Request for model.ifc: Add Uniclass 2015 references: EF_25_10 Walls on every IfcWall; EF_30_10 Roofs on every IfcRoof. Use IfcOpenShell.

First a look at what the model holds.

```python
import ifcopenshell

model = ifcopenshell.open("model.ifc")
print(model.schema)
print("classifications:", [c.Name for c in model.by_type("IfcClassification")])
for ifc_class in ("IfcDoor", "IfcRoof", "IfcStair", "IfcWall", "IfcWindow"):
    print(ifc_class, len(model.by_type(ifc_class)))
```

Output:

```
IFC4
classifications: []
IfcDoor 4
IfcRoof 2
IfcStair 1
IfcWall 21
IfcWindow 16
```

```python
import ifcopenshell
import ifcopenshell.api.classification

model = ifcopenshell.open("model.ifc")

system = ifcopenshell.api.classification.add_classification(model, classification="Uniclass 2015")

codes = {
    "IfcWall": ("EF_25_10", "Walls"),
    "IfcRoof": ("EF_30_10", "Roofs"),
}
for ifc_class, (code, name) in codes.items():
    products = model.by_type(ifc_class)
    ifcopenshell.api.classification.add_reference(
        model, products=products, classification=system, identification=code, name=name
    )
    print(code, len(products))

model.write("model_edited.ifc")
```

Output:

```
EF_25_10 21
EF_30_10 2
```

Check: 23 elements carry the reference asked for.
